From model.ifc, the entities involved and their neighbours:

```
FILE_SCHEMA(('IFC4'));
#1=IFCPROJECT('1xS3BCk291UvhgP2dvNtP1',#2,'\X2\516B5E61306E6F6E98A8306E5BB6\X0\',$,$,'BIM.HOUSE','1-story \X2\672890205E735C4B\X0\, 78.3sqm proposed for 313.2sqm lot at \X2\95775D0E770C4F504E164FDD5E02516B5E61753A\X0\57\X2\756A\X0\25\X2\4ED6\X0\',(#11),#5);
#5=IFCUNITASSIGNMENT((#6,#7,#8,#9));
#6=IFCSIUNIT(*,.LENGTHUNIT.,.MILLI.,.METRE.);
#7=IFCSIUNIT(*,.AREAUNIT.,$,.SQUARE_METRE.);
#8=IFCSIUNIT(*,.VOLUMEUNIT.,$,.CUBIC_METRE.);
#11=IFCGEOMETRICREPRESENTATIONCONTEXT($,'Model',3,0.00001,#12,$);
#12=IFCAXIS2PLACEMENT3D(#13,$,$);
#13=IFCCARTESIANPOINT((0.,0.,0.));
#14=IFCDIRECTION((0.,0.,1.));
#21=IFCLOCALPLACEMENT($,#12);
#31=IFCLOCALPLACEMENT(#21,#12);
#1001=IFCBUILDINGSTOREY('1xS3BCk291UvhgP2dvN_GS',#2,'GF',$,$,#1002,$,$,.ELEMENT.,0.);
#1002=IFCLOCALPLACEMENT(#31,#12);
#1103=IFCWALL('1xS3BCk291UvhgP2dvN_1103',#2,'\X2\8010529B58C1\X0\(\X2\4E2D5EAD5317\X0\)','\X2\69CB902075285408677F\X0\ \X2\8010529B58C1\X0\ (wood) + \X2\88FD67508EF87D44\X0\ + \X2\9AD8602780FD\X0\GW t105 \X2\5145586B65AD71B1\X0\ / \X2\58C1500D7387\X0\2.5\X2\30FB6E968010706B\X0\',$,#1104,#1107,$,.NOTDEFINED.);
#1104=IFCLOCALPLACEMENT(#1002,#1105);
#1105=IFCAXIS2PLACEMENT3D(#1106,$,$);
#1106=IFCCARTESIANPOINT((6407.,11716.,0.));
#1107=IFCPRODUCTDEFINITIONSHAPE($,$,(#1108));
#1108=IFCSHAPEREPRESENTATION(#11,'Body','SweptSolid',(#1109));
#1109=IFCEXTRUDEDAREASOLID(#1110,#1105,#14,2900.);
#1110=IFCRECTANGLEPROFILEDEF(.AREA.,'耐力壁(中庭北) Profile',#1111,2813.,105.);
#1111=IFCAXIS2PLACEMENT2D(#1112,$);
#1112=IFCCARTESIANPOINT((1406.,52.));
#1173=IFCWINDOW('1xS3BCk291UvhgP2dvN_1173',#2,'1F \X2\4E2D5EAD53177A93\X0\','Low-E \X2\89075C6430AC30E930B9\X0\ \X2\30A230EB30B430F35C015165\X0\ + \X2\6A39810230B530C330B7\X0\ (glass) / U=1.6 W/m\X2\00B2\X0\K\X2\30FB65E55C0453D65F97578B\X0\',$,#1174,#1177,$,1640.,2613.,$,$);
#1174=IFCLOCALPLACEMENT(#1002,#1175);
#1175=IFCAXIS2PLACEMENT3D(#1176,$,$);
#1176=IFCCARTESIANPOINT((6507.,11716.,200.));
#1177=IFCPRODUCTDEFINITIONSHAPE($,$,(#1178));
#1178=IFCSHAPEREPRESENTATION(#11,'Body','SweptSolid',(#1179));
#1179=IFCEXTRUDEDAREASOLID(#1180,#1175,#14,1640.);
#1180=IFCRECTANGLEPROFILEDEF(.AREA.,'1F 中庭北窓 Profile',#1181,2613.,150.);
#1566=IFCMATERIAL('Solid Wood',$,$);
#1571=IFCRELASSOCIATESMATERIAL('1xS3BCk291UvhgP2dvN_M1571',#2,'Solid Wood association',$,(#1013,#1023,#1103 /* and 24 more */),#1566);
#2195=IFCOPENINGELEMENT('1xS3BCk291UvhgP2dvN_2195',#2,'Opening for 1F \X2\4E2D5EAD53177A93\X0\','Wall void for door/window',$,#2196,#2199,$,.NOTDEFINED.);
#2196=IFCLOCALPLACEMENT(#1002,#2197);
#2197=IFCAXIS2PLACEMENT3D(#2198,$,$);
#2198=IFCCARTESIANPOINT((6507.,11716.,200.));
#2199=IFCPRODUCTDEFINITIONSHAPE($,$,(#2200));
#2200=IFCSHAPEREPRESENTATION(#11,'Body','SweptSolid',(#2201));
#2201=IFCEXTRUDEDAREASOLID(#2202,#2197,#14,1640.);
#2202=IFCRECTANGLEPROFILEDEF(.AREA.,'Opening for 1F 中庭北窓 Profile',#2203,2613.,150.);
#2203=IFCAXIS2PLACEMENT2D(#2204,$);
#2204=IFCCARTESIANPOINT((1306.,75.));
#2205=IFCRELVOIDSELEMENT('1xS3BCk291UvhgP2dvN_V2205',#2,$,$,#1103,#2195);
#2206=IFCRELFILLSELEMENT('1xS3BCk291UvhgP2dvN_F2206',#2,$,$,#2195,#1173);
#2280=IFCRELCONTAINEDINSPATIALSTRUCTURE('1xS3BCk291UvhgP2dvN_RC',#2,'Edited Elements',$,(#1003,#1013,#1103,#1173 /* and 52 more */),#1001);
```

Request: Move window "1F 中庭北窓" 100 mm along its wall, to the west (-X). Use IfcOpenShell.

```python
import ifcopenshell
import ifcopenshell.api.geometry
import ifcopenshell.util.placement
import ifcopenshell.util.unit

model = ifcopenshell.open("model.ifc")
unit_scale = ifcopenshell.util.unit.calculate_unit_scale(model)

window = model.by_guid("1xS3BCk291UvhgP2dvN_1173")
opening = window.FillsVoids[0].RelatingOpeningElement
wall = opening.VoidsElements[0].RelatingBuildingElement

wall_matrix = ifcopenshell.util.placement.get_local_placement(wall.ObjectPlacement)
shift = wall_matrix[:3, 0] * -0.1 / unit_scale
before = ifcopenshell.util.placement.get_local_placement(window.ObjectPlacement)[:3, 3].copy()

# The window is not placed relative to its opening, so move both.
for product in (opening, window):
    matrix = ifcopenshell.util.placement.get_local_placement(product.ObjectPlacement)
    matrix[:3, 3] += shift
    ifcopenshell.api.geometry.edit_object_placement(model, product=product, matrix=matrix, is_si=False)

after = ifcopenshell.util.placement.get_local_placement(window.ObjectPlacement)[:3, 3]
print("window moved by", (after - before).round(3) + 0.0)

model.write("model_v2.ifc")
```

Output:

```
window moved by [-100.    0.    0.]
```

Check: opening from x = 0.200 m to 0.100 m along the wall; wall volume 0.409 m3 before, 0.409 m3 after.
